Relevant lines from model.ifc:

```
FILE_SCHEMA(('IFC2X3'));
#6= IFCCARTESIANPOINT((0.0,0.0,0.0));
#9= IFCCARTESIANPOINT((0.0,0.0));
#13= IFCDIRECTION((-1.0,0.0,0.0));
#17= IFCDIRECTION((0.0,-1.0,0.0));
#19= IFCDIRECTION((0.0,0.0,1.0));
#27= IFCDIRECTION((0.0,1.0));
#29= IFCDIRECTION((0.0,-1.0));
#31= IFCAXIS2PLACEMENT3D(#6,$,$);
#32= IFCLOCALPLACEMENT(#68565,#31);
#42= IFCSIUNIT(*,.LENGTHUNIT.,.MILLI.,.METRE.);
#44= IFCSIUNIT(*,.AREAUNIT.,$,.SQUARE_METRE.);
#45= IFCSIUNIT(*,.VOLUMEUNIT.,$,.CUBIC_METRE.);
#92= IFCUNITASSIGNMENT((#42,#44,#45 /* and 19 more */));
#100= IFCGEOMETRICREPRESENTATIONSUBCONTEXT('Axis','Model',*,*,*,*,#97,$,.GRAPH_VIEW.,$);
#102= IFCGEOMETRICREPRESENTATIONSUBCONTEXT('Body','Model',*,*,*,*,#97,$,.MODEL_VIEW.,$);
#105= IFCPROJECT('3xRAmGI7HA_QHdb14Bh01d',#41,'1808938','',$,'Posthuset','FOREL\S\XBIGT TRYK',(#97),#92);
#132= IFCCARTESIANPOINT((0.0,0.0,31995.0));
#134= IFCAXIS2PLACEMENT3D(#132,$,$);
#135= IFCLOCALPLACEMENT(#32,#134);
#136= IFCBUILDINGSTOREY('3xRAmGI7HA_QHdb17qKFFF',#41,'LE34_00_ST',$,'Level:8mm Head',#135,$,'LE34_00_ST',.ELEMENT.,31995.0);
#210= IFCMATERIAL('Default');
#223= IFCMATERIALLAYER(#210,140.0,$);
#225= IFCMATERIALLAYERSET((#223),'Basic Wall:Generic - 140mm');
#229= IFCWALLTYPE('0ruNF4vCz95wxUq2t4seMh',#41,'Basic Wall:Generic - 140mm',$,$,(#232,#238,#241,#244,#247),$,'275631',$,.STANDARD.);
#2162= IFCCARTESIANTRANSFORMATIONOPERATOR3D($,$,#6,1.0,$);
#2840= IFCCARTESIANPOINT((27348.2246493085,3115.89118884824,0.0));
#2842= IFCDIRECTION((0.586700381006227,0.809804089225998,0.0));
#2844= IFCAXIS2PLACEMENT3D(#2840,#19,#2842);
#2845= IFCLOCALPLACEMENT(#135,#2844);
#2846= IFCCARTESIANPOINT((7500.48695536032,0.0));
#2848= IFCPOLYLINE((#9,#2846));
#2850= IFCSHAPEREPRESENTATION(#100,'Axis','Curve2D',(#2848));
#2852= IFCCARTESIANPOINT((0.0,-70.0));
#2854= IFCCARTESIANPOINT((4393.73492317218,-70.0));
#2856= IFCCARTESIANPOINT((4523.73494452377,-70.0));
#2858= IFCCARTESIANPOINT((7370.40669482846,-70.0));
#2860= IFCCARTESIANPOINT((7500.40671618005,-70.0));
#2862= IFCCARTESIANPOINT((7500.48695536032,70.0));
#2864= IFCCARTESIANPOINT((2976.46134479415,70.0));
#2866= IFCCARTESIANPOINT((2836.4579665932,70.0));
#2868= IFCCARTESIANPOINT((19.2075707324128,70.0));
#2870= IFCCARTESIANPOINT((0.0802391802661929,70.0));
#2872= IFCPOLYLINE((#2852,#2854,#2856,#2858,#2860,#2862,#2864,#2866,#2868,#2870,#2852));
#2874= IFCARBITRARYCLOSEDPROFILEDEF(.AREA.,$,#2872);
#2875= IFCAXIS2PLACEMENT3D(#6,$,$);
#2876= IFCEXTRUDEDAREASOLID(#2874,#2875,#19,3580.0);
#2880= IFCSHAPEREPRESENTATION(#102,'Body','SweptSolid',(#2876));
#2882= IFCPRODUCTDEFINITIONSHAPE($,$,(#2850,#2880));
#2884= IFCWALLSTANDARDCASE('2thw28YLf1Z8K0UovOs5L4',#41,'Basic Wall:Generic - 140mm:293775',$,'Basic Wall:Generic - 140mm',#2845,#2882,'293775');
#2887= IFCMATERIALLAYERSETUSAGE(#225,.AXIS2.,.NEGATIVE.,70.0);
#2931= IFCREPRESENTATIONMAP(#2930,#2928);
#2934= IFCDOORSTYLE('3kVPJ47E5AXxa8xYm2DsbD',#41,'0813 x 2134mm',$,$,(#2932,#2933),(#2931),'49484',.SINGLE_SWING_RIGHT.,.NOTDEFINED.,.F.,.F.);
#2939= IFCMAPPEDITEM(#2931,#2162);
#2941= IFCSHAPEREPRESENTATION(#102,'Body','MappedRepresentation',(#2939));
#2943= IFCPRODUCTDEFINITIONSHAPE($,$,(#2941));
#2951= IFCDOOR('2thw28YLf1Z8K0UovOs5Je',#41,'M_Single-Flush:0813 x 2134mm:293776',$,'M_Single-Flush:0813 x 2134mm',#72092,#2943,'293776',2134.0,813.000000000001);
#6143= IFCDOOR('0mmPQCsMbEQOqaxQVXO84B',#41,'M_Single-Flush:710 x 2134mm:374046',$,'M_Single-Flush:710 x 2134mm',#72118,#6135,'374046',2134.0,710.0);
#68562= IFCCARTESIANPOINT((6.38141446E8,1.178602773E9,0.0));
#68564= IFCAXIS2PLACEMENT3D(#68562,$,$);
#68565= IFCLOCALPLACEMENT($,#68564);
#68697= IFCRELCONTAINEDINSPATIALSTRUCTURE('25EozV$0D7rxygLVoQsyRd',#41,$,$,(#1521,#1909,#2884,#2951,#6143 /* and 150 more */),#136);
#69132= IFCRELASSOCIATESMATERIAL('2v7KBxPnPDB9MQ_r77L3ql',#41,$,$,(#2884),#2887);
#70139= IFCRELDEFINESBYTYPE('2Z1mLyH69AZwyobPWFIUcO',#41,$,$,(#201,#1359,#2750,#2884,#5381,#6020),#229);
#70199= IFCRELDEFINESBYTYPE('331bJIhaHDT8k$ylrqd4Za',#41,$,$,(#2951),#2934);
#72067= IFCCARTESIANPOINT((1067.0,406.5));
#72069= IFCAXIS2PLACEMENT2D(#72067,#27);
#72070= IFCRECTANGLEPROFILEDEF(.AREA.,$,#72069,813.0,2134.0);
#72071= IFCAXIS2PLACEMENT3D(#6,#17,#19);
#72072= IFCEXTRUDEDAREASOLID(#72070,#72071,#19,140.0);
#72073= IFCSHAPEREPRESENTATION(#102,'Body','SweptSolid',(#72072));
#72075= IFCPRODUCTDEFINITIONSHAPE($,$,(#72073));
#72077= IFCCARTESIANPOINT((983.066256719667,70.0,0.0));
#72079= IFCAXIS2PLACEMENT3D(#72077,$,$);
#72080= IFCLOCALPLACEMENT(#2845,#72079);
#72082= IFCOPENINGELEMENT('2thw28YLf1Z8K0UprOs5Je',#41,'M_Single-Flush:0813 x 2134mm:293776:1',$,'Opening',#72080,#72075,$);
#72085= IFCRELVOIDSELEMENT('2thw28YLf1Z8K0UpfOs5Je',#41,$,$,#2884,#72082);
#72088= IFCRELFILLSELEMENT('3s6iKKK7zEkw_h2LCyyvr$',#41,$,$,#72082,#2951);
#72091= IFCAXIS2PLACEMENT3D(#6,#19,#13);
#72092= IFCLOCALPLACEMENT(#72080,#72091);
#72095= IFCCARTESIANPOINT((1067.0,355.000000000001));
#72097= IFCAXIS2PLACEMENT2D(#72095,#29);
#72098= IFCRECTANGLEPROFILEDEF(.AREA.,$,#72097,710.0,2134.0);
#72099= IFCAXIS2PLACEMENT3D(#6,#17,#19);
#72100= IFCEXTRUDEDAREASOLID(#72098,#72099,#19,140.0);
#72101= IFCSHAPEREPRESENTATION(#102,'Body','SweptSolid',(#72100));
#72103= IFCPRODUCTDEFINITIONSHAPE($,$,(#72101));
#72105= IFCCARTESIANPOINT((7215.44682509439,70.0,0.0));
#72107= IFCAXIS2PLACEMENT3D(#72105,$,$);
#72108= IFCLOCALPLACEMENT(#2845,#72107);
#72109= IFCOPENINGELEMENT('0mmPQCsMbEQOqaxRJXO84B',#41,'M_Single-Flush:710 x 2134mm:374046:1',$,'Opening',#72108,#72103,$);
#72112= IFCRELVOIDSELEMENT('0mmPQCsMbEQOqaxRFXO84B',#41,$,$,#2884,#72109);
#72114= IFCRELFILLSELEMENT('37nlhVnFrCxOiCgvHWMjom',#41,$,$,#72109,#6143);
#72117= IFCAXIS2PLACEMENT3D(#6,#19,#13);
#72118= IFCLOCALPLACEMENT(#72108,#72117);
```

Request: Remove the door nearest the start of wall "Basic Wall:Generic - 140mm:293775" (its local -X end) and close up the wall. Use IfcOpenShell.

```python
import ifcopenshell
import ifcopenshell.api.feature
import ifcopenshell.api.root
import ifcopenshell.geom
import ifcopenshell.util.shape

model = ifcopenshell.open("model.ifc")
settings = ifcopenshell.geom.settings()


def volume(element):
    """Net volume in cubic metres, openings subtracted."""
    shape = ifcopenshell.geom.create_shape(settings, element)
    return ifcopenshell.util.shape.get_volume(shape.geometry)


door = model.by_guid("2thw28YLf1Z8K0UovOs5Je")
opening = door.FillsVoids[0].RelatingOpeningElement
wall = opening.VoidsElements[0].RelatingBuildingElement
before = volume(wall)

ifcopenshell.api.root.remove_product(model, product=door)
ifcopenshell.api.feature.remove_feature(model, feature=opening)

after = volume(wall)

print(f"wall volume {before:.3f} -> {after:.3f} m3")

model.write("model_v2.ifc")
```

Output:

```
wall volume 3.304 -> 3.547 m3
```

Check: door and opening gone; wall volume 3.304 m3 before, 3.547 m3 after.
